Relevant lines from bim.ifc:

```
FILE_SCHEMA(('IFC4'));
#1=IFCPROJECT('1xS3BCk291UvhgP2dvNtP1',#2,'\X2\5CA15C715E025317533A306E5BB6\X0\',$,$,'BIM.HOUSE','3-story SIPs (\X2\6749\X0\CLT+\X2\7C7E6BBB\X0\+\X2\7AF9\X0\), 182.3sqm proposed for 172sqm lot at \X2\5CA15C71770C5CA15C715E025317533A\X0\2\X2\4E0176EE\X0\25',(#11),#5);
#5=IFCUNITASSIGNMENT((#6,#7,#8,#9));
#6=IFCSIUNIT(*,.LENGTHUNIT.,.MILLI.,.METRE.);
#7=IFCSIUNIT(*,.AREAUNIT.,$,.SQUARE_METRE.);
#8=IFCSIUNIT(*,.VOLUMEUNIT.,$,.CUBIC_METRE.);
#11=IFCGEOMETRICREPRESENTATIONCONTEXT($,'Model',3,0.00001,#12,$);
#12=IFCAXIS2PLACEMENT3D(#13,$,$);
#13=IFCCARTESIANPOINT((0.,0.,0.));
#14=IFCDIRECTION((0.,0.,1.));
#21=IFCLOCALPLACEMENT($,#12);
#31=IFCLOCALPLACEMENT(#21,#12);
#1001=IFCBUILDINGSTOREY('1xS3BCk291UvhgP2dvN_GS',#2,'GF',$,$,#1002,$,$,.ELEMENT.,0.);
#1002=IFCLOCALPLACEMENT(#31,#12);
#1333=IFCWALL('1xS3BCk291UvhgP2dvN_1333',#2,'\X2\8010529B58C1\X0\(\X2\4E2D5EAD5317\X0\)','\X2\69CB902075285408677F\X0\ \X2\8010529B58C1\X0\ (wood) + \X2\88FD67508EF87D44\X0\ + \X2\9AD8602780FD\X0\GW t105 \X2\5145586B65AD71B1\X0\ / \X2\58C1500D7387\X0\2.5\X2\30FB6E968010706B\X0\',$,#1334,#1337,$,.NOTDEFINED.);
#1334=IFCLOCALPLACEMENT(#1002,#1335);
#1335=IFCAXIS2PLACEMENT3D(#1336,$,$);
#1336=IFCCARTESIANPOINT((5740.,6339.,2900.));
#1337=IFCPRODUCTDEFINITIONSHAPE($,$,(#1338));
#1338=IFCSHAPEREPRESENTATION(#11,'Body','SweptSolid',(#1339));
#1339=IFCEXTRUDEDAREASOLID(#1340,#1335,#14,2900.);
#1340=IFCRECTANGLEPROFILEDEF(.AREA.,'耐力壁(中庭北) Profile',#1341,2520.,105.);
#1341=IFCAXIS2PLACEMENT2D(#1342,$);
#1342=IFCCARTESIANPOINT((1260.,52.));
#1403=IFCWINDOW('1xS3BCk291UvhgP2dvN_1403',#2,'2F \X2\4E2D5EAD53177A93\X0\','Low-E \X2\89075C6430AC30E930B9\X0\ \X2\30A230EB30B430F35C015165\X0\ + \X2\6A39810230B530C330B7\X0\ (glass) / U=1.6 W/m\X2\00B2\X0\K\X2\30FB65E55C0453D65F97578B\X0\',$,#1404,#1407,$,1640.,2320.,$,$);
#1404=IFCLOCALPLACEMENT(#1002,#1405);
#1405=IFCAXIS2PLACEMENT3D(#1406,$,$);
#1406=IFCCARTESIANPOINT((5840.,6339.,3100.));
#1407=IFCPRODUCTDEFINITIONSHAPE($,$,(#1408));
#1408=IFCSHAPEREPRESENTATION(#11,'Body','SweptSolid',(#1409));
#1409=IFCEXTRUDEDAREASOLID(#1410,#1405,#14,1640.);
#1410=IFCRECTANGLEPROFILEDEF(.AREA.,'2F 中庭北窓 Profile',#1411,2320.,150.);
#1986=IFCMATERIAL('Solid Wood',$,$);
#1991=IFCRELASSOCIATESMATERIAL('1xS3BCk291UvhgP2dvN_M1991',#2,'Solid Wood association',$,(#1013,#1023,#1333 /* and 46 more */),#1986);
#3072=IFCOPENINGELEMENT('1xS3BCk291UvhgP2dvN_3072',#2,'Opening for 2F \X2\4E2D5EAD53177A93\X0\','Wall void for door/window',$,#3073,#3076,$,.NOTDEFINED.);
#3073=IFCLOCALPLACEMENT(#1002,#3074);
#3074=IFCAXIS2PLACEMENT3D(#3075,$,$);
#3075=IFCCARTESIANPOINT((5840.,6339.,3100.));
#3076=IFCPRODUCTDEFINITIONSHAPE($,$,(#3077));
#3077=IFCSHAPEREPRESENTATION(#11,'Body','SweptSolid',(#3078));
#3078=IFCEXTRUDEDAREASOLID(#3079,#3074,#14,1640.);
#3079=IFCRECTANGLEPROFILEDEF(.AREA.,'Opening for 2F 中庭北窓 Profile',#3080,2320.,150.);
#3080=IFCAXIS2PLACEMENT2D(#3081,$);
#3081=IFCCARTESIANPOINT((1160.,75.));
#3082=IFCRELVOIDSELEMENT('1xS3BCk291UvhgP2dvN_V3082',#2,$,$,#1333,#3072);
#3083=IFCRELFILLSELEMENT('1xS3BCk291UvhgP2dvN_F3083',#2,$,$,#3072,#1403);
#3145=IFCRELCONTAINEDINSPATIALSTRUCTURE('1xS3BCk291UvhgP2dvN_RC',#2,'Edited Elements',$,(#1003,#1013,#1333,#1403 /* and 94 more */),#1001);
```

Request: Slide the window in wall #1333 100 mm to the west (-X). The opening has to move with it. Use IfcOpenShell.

```python
import ifcopenshell
import ifcopenshell.api.geometry
import ifcopenshell.util.placement

model = ifcopenshell.open("bim.ifc")

window = model.by_guid("1xS3BCk291UvhgP2dvN_1403")
opening = window.FillsVoids[0].RelatingOpeningElement
wall = opening.VoidsElements[0].RelatingBuildingElement

wall_matrix = ifcopenshell.util.placement.get_local_placement(wall.ObjectPlacement)
shift = wall_matrix[:3, 0] * -100.0
before = ifcopenshell.util.placement.get_local_placement(window.ObjectPlacement)[:3, 3].copy()

# The window is not placed relative to its opening, so move both.
for product in (opening, window):
    matrix = ifcopenshell.util.placement.get_local_placement(product.ObjectPlacement)
    matrix[:3, 3] += shift
    ifcopenshell.api.geometry.edit_object_placement(model, product=product, matrix=matrix, is_si=False)

after = ifcopenshell.util.placement.get_local_placement(window.ObjectPlacement)[:3, 3]
print("window moved by", (after - before).round(3) + 0.0)

model.write("bim_rev.ifc")
```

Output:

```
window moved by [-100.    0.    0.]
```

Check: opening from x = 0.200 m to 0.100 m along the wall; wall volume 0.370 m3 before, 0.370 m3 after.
